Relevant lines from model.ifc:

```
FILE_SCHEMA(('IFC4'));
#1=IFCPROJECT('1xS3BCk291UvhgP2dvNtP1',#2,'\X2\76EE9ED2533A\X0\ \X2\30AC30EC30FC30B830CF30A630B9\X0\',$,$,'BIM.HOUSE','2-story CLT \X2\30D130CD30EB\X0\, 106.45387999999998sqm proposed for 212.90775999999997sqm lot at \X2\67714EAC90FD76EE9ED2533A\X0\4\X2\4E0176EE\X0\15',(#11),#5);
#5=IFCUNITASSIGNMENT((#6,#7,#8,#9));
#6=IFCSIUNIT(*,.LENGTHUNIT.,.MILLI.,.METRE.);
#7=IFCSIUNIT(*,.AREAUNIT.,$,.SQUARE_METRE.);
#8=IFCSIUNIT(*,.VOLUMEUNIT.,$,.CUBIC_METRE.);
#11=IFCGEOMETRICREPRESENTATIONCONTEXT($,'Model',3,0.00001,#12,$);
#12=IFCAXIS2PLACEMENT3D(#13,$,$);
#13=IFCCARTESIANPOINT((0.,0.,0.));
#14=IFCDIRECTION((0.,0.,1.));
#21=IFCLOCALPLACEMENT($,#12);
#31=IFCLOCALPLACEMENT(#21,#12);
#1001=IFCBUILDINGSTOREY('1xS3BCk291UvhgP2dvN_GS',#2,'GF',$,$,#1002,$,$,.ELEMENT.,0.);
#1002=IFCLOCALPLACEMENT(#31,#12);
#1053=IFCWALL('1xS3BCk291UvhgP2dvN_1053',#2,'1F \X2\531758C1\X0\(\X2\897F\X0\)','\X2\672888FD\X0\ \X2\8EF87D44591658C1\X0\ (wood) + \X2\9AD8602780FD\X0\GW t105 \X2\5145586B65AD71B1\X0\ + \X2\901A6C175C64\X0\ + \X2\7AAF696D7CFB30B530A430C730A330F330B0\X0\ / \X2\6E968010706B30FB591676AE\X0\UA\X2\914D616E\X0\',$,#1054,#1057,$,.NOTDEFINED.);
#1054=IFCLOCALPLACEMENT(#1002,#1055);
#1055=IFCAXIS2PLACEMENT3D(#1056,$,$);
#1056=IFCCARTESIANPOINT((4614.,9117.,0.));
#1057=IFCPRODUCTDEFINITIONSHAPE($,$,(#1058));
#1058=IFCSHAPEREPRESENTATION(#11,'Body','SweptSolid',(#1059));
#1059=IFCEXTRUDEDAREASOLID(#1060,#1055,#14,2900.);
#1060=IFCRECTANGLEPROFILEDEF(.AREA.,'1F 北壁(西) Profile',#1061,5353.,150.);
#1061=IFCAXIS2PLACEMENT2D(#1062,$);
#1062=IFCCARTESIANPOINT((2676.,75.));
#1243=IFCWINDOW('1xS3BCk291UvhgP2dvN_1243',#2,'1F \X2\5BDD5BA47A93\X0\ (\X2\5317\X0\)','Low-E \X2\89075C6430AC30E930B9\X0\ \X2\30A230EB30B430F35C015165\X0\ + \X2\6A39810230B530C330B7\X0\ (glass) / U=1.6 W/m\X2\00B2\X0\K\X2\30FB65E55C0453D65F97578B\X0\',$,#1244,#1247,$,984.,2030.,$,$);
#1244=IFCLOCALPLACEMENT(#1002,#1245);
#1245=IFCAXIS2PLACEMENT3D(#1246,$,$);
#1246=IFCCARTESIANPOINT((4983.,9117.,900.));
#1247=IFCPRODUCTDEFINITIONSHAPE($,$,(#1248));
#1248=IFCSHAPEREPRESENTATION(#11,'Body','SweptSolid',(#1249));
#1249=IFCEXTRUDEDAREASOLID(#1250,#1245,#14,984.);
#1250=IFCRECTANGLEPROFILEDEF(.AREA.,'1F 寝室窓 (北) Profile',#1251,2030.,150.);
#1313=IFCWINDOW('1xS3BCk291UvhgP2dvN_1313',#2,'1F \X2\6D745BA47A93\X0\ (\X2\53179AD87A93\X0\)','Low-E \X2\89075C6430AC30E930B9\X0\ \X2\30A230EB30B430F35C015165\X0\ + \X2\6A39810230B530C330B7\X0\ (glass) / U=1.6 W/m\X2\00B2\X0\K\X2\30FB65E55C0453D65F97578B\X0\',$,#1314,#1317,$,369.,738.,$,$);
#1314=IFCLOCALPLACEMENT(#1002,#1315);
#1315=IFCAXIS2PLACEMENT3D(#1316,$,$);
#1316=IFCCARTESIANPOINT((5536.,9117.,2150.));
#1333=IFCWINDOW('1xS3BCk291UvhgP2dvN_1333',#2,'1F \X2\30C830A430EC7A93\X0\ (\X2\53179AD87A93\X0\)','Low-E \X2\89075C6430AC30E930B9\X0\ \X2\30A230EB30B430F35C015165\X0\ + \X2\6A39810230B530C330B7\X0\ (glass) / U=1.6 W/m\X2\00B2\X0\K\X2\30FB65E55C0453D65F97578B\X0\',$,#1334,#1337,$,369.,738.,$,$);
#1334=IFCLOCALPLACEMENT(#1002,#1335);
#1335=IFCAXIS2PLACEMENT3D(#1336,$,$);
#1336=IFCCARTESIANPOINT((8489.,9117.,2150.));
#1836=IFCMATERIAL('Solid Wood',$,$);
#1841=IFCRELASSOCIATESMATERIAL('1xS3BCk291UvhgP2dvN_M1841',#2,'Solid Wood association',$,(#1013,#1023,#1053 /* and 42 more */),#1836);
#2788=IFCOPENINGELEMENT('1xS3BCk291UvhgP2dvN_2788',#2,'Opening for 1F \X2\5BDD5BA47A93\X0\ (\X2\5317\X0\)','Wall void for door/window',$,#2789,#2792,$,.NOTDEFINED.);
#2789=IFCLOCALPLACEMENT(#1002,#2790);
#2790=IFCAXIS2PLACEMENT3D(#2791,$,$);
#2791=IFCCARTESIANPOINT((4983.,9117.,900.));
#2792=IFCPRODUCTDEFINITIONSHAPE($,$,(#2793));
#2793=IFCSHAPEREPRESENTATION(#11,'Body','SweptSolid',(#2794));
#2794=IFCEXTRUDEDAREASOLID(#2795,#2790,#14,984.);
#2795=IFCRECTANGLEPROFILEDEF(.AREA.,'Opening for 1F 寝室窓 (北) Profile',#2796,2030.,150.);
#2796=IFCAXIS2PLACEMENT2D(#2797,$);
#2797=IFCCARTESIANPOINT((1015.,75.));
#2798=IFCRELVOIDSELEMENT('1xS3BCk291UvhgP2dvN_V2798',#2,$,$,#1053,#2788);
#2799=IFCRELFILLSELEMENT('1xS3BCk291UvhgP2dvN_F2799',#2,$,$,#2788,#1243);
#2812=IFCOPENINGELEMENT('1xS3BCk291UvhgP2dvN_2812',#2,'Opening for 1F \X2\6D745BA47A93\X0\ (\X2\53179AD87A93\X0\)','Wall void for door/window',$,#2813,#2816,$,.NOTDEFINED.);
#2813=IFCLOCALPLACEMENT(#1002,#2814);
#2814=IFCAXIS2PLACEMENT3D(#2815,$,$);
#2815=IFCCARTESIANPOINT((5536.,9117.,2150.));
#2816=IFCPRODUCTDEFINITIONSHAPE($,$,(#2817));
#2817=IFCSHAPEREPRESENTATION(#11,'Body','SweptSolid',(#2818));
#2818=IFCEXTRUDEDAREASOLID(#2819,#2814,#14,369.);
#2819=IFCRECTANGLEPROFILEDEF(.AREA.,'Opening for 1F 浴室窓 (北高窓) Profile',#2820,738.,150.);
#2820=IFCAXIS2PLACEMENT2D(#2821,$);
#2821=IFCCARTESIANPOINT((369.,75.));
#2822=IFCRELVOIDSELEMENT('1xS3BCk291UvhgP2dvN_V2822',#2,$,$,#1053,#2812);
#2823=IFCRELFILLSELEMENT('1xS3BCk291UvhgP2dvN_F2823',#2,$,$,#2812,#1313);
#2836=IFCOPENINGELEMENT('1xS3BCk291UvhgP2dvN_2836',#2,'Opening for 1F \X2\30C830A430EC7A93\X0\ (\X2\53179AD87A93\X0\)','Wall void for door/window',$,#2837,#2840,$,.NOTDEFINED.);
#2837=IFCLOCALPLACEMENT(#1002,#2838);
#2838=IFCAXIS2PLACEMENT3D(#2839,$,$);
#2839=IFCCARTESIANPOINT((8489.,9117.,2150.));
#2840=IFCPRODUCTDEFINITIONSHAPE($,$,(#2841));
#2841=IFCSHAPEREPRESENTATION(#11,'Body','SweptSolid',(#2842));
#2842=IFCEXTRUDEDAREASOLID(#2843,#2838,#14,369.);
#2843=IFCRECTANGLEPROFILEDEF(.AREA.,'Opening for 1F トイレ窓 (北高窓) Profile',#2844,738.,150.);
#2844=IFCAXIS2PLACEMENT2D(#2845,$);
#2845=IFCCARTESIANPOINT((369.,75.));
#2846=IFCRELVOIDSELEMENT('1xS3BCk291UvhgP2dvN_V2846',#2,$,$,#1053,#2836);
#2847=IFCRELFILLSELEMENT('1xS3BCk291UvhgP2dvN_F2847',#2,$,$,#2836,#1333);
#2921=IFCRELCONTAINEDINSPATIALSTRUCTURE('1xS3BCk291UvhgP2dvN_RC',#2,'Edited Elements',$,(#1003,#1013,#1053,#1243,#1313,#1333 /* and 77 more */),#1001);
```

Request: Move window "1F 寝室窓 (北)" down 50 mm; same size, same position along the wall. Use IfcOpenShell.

```python
import numpy as np
import ifcopenshell
import ifcopenshell.api.geometry
import ifcopenshell.util.placement
import ifcopenshell.util.unit

model = ifcopenshell.open("model.ifc")
unit_scale = ifcopenshell.util.unit.calculate_unit_scale(model)

window = model.by_id(1243)
opening = window.FillsVoids[0].RelatingOpeningElement
dz = -50.0

shift = np.array([0.0, 0.0, dz])
# The window is not placed relative to its opening, so move both.
for product in (opening, window):
    matrix = ifcopenshell.util.placement.get_local_placement(product.ObjectPlacement)
    matrix[:3, 3] += shift
    ifcopenshell.api.geometry.edit_object_placement(model, product=product, matrix=matrix, is_si=False)

print(f"moved by {dz * unit_scale:+.3f} m")

model.write("model-out.ifc")
```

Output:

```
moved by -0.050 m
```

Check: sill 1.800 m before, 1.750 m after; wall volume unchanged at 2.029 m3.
